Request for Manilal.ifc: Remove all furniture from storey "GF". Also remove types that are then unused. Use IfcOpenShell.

First a look at what the model holds.

```python
import ifcopenshell
import ifcopenshell.util.element

model = ifcopenshell.open("Manilal.ifc")
print(model.schema)
storey = next(s for s in model.by_type("IfcBuildingStorey") if s.Name == "GF")
furniture = [e for e in ifcopenshell.util.element.get_decomposition(storey) if e.is_a("IfcFurnishingElement")]
seen = {}
for e in furniture:
    element_type = ifcopenshell.util.element.get_type(e)
    name = element_type.Name if element_type not in (None, e) else None
    seen[name] = seen.get(name, 0) + 1
for name, count in sorted(seen.items(), key=str):
    print(count, "x", name)
```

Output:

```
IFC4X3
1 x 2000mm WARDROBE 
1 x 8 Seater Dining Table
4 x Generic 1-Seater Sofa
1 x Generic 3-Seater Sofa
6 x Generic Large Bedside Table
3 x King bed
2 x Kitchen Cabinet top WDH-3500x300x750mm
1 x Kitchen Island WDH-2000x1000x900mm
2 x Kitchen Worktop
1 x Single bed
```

```python
import ifcopenshell
import ifcopenshell.api.root
import ifcopenshell.util.element

model = ifcopenshell.open("Manilal.ifc")

storey = next(s for s in model.by_type("IfcBuildingStorey") if s.Name == "GF")
furniture = [e for e in ifcopenshell.util.element.get_decomposition(storey) if e.is_a("IfcFurnishingElement")]
types = {ifcopenshell.util.element.get_type(e) for e in furniture} - {None, *furniture}

for e in furniture:
    ifcopenshell.api.root.remove_product(model, product=e)
print(len(furniture), "removed")

unused = [t for t in types if not ifcopenshell.util.element.get_types(t)]
for t in unused:
    ifcopenshell.api.root.remove_product(model, product=t)
print(len(unused), "unused types removed")

model.write("Manilal_rev.ifc")
```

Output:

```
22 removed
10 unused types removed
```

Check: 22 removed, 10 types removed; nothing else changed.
